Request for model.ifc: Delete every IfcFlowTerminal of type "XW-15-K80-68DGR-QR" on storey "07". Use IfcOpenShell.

First a look at what the model holds.

```python
import ifcopenshell
import ifcopenshell.util.element

model = ifcopenshell.open("model.ifc")
print(model.schema)
storey = next(s for s in model.by_type("IfcBuildingStorey") if s.Name == "07")
terminals = [e for e in ifcopenshell.util.element.get_decomposition(storey) if e.is_a("IfcFlowTerminal")]
seen = {}
for e in terminals:
    element_type = ifcopenshell.util.element.get_type(e)
    name = element_type.Name if element_type not in (None, e) else None
    seen[name] = seen.get(name, 0) + 1
for name, count in sorted(seen.items(), key=str):
    print(count, "x", name)
```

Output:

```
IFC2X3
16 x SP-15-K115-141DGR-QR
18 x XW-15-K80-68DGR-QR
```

```python
import ifcopenshell
import ifcopenshell.api.root
import ifcopenshell.util.element

model = ifcopenshell.open("model.ifc")

storey = next(s for s in model.by_type("IfcBuildingStorey") if s.Name == "07")
terminals = [e for e in ifcopenshell.util.element.get_decomposition(storey) if e.is_a("IfcFlowTerminal")]
targets = [e for e in terminals if (t := ifcopenshell.util.element.get_type(e)) not in (None, e) and t.Name == "XW-15-K80-68DGR-QR"]

for e in targets:
    ifcopenshell.api.root.remove_product(model, product=e)
print(len(targets), "removed")

model.write("model-out.ifc")
```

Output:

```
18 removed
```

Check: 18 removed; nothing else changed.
